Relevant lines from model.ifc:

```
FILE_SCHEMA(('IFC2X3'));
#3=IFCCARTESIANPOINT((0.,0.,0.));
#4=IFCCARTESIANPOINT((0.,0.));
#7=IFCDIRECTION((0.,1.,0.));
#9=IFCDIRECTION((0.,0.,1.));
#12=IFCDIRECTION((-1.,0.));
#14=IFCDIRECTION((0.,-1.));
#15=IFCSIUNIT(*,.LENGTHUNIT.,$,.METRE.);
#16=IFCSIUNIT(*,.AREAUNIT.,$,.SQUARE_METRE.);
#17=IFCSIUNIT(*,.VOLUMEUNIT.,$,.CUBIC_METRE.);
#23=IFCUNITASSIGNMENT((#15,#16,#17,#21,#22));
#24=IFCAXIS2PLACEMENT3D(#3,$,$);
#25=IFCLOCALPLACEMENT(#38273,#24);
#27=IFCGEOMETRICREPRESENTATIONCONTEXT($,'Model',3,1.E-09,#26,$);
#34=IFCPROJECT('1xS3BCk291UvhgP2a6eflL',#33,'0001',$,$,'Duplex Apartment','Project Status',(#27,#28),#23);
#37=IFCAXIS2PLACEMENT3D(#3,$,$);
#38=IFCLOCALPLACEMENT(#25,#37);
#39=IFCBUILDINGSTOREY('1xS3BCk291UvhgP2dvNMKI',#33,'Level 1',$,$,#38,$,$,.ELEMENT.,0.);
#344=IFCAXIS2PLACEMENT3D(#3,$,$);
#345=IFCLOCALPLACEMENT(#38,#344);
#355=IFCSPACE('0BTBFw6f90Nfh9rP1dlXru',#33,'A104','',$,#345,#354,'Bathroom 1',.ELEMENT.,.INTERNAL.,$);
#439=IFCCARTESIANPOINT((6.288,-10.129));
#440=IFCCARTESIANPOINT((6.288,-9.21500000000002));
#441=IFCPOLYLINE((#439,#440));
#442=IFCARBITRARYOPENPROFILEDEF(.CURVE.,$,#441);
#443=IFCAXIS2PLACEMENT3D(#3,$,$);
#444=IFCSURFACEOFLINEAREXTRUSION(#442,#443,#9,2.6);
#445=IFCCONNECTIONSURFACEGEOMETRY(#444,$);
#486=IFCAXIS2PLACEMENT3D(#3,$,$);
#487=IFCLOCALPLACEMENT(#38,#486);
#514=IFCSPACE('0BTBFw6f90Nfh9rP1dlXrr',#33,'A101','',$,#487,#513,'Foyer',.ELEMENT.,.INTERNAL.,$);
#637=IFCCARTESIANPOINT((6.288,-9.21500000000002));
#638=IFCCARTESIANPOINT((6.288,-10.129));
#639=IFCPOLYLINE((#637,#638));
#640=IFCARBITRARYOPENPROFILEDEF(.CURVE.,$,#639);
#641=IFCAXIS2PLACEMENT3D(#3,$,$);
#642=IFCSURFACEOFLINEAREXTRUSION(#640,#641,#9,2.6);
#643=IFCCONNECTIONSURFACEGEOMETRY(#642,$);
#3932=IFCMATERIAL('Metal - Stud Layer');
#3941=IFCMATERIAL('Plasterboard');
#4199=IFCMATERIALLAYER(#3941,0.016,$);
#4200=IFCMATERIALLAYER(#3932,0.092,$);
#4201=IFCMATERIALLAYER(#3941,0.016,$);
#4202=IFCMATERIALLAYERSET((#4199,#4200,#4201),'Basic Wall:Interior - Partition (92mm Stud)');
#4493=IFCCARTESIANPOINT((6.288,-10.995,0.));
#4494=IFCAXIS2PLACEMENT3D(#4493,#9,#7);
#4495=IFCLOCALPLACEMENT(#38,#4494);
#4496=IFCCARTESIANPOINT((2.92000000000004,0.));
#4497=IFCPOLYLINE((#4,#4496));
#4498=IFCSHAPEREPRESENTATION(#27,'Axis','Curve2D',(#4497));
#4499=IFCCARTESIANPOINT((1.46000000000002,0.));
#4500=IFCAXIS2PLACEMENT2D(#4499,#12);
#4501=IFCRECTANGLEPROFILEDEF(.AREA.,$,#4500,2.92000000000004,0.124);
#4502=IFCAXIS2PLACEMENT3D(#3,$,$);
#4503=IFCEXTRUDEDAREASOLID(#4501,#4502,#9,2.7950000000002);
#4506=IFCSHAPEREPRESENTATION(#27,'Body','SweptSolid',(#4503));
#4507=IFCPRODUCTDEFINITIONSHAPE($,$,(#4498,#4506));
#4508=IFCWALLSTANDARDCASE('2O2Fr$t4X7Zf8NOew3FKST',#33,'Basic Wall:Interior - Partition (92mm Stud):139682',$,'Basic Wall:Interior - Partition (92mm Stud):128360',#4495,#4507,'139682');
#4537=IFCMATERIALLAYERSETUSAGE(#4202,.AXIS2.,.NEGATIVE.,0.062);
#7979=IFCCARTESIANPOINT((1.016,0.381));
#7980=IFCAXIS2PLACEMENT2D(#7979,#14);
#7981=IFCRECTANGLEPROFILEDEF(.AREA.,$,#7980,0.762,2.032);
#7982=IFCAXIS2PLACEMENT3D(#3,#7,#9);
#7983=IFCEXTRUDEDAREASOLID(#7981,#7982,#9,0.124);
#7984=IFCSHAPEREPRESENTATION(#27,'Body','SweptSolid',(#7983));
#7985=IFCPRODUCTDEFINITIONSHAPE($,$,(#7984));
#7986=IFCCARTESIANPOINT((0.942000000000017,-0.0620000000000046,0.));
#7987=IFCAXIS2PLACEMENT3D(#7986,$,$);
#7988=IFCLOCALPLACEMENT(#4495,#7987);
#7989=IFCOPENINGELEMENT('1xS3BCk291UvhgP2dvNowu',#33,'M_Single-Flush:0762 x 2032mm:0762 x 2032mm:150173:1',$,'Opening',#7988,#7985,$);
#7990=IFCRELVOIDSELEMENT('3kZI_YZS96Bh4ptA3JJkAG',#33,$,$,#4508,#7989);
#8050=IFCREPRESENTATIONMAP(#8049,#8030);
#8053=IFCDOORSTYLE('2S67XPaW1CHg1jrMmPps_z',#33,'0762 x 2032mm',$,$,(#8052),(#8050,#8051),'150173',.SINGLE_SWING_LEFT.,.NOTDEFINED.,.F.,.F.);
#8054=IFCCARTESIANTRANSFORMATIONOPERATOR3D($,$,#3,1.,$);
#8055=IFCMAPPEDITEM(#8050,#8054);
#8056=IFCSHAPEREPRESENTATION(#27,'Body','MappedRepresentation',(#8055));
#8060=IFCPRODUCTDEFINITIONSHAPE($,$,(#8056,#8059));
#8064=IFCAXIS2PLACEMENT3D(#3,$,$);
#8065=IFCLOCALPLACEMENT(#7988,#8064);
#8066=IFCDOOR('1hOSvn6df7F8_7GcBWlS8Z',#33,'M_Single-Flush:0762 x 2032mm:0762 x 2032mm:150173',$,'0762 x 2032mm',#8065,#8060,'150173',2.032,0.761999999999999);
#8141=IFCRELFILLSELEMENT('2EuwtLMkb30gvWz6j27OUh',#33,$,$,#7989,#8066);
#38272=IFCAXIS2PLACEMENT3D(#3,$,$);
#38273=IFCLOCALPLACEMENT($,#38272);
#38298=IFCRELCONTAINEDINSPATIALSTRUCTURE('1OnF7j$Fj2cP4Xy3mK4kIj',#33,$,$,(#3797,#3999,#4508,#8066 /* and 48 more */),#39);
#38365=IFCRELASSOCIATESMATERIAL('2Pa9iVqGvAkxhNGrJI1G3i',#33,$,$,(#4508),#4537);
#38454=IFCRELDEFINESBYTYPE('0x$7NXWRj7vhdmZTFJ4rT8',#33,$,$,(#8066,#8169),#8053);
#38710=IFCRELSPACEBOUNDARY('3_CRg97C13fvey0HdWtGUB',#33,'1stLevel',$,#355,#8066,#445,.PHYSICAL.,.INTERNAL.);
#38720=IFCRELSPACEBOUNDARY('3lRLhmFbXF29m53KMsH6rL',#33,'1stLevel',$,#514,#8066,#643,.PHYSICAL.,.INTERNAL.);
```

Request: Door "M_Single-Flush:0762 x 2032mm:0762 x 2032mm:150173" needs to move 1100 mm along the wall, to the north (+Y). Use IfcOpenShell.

```python
import numpy as np
import ifcopenshell
import ifcopenshell.api.geometry
import ifcopenshell.util.placement

model = ifcopenshell.open("model.ifc")

door = model.by_id(8066)
opening = door.FillsVoids[0].RelatingOpeningElement
wall = opening.VoidsElements[0].RelatingBuildingElement

wall_matrix = ifcopenshell.util.placement.get_local_placement(wall.ObjectPlacement)
shift = wall_matrix[:3, 0] * 1.1
before = ifcopenshell.util.placement.get_local_placement(door.ObjectPlacement)[:3, 3].copy()

# The door is placed relative to its opening, so it follows when the opening moves.
matrix = ifcopenshell.util.placement.get_local_placement(opening.ObjectPlacement)
matrix[:3, 3] += shift
ifcopenshell.api.geometry.edit_object_placement(
    model, product=opening, matrix=matrix, is_si=False, should_transform_children=True
)

# Space boundary surfaces are stored in each space's coordinates; move them too.
for rel in door.ProvidesBoundaries:
    if not rel.ConnectionGeometry:
        continue
    surface = rel.ConnectionGeometry.SurfaceOnRelatingElement
    space_matrix = ifcopenshell.util.placement.get_local_placement(rel.RelatingSpace.ObjectPlacement)
    point = np.array(surface.Position.Location.Coordinates) + space_matrix[:3, :3].T @ shift
    surface.Position = model.createIfcAxis2Placement3D(
        model.createIfcCartesianPoint(point.tolist()), surface.Position.Axis, surface.Position.RefDirection
    )

after = ifcopenshell.util.placement.get_local_placement(door.ObjectPlacement)[:3, 3]
print("door moved by", (after - before).round(3) + 0.0)

model.write("model-out.ifc")
```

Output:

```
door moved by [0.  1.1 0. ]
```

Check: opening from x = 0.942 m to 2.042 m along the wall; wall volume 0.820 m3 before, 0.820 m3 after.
